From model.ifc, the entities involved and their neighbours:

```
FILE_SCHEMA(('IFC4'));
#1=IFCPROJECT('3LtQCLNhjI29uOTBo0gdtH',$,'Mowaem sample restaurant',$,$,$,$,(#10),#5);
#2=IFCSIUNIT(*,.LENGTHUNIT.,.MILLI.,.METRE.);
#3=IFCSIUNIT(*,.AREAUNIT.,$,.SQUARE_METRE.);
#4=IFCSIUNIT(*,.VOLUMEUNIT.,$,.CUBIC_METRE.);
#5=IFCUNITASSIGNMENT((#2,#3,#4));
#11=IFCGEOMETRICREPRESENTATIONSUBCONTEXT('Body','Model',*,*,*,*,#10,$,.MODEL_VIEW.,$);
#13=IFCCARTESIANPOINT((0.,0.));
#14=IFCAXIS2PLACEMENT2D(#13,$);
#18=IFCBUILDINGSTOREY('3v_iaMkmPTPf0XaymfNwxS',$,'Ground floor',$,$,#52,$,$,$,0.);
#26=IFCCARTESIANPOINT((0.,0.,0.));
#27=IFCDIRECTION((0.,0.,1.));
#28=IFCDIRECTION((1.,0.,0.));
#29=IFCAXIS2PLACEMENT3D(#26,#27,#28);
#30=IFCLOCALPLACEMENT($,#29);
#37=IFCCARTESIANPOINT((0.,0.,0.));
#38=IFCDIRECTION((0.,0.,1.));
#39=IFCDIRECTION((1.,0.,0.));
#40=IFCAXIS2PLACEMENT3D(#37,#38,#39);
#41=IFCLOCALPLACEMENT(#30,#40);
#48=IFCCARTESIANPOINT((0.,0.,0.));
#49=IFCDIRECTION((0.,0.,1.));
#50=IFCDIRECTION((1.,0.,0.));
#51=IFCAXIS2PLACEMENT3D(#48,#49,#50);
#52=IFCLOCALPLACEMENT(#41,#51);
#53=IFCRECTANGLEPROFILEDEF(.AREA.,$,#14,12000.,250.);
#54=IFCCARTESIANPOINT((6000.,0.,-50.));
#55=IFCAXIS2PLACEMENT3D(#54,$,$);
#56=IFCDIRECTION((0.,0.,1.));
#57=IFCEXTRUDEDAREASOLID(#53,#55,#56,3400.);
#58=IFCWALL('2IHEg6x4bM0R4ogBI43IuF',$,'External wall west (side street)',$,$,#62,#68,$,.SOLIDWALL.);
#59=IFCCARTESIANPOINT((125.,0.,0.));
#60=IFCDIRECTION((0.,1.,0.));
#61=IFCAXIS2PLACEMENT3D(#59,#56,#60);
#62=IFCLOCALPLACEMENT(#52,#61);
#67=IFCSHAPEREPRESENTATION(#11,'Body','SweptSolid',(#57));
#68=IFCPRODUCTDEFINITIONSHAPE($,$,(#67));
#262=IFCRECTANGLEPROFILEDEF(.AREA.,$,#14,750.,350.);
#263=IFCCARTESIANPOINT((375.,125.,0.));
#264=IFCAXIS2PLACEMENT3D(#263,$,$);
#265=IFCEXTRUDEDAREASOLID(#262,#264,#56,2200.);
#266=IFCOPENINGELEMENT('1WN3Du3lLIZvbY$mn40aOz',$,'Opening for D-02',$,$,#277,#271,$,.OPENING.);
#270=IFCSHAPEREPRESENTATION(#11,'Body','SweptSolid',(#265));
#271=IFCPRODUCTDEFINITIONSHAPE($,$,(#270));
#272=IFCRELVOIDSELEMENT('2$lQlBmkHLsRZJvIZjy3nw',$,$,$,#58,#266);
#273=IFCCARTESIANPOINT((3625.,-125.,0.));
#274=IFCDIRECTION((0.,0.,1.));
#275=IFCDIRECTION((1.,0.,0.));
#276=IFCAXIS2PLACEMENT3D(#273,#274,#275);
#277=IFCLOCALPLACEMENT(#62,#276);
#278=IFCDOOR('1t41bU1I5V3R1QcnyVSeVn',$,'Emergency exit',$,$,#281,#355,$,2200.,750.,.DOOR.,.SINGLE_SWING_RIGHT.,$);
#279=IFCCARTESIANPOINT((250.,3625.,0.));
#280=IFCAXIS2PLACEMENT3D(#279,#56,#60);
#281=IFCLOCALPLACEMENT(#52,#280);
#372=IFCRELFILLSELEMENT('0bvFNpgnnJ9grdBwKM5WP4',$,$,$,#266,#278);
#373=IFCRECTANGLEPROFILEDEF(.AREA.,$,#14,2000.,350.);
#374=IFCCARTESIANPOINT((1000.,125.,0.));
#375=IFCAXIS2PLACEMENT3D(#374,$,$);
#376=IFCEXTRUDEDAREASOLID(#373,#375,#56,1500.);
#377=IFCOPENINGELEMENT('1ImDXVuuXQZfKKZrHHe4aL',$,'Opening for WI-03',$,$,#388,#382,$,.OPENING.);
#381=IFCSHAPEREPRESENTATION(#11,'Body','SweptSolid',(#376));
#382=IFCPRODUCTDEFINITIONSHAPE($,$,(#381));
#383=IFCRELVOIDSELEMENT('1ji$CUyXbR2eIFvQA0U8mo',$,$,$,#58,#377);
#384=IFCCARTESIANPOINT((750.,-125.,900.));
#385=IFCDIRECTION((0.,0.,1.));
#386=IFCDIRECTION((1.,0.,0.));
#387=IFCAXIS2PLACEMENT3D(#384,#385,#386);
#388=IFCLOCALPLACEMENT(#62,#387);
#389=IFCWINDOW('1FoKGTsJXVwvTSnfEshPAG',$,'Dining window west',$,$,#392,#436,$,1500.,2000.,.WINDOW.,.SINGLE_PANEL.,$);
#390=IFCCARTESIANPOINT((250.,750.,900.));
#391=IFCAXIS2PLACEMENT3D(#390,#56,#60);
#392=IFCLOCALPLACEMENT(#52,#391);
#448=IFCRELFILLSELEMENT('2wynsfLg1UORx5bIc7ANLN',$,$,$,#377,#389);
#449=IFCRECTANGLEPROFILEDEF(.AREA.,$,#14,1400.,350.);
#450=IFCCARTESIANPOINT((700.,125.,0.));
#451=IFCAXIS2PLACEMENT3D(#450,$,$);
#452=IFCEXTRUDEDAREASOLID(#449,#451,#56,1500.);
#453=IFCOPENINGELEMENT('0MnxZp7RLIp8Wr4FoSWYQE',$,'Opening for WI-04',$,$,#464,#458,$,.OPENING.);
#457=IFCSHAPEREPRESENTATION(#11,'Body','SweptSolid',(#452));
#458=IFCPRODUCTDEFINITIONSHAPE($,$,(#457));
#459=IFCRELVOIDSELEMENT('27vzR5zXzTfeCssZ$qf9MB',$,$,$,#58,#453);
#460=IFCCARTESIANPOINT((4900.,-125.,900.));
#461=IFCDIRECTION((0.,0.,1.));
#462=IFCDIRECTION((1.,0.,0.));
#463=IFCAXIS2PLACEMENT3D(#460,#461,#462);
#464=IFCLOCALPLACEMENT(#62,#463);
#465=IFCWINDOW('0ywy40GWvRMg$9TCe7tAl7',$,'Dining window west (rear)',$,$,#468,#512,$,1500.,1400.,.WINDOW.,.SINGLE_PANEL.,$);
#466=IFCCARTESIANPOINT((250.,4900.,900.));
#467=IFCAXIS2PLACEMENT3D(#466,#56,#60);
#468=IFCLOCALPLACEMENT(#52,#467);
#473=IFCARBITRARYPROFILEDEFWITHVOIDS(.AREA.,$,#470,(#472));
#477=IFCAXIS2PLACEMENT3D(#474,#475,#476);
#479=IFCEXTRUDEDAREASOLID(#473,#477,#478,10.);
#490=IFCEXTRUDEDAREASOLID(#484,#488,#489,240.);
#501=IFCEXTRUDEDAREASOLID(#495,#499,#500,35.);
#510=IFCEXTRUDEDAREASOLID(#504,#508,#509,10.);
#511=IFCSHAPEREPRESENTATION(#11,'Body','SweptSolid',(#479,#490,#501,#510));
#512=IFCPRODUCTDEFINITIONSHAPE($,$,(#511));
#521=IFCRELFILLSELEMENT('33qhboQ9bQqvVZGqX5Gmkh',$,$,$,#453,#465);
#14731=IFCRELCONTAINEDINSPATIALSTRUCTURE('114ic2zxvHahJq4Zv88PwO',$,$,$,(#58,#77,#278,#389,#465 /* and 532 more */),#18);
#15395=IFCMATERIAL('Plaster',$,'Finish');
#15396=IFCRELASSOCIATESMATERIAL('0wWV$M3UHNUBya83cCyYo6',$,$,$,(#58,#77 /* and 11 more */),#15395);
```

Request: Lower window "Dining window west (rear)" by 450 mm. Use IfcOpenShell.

```python
import numpy as np
import ifcopenshell
import ifcopenshell.api.geometry
import ifcopenshell.util.placement
import ifcopenshell.util.unit

model = ifcopenshell.open("model.ifc")
unit_scale = ifcopenshell.util.unit.calculate_unit_scale(model)

window = model.by_id(465)
opening = window.FillsVoids[0].RelatingOpeningElement
dz = -0.45 / unit_scale

shift = np.array([0.0, 0.0, dz])
# The window is not placed relative to its opening, so move both.
for product in (opening, window):
    matrix = ifcopenshell.util.placement.get_local_placement(product.ObjectPlacement)
    matrix[:3, 3] += shift
    ifcopenshell.api.geometry.edit_object_placement(model, product=product, matrix=matrix, is_si=False)

print(f"moved by {dz * unit_scale:+.3f} m")

model.write("model_updated.ifc")
```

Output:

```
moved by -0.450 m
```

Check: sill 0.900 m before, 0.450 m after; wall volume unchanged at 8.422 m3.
